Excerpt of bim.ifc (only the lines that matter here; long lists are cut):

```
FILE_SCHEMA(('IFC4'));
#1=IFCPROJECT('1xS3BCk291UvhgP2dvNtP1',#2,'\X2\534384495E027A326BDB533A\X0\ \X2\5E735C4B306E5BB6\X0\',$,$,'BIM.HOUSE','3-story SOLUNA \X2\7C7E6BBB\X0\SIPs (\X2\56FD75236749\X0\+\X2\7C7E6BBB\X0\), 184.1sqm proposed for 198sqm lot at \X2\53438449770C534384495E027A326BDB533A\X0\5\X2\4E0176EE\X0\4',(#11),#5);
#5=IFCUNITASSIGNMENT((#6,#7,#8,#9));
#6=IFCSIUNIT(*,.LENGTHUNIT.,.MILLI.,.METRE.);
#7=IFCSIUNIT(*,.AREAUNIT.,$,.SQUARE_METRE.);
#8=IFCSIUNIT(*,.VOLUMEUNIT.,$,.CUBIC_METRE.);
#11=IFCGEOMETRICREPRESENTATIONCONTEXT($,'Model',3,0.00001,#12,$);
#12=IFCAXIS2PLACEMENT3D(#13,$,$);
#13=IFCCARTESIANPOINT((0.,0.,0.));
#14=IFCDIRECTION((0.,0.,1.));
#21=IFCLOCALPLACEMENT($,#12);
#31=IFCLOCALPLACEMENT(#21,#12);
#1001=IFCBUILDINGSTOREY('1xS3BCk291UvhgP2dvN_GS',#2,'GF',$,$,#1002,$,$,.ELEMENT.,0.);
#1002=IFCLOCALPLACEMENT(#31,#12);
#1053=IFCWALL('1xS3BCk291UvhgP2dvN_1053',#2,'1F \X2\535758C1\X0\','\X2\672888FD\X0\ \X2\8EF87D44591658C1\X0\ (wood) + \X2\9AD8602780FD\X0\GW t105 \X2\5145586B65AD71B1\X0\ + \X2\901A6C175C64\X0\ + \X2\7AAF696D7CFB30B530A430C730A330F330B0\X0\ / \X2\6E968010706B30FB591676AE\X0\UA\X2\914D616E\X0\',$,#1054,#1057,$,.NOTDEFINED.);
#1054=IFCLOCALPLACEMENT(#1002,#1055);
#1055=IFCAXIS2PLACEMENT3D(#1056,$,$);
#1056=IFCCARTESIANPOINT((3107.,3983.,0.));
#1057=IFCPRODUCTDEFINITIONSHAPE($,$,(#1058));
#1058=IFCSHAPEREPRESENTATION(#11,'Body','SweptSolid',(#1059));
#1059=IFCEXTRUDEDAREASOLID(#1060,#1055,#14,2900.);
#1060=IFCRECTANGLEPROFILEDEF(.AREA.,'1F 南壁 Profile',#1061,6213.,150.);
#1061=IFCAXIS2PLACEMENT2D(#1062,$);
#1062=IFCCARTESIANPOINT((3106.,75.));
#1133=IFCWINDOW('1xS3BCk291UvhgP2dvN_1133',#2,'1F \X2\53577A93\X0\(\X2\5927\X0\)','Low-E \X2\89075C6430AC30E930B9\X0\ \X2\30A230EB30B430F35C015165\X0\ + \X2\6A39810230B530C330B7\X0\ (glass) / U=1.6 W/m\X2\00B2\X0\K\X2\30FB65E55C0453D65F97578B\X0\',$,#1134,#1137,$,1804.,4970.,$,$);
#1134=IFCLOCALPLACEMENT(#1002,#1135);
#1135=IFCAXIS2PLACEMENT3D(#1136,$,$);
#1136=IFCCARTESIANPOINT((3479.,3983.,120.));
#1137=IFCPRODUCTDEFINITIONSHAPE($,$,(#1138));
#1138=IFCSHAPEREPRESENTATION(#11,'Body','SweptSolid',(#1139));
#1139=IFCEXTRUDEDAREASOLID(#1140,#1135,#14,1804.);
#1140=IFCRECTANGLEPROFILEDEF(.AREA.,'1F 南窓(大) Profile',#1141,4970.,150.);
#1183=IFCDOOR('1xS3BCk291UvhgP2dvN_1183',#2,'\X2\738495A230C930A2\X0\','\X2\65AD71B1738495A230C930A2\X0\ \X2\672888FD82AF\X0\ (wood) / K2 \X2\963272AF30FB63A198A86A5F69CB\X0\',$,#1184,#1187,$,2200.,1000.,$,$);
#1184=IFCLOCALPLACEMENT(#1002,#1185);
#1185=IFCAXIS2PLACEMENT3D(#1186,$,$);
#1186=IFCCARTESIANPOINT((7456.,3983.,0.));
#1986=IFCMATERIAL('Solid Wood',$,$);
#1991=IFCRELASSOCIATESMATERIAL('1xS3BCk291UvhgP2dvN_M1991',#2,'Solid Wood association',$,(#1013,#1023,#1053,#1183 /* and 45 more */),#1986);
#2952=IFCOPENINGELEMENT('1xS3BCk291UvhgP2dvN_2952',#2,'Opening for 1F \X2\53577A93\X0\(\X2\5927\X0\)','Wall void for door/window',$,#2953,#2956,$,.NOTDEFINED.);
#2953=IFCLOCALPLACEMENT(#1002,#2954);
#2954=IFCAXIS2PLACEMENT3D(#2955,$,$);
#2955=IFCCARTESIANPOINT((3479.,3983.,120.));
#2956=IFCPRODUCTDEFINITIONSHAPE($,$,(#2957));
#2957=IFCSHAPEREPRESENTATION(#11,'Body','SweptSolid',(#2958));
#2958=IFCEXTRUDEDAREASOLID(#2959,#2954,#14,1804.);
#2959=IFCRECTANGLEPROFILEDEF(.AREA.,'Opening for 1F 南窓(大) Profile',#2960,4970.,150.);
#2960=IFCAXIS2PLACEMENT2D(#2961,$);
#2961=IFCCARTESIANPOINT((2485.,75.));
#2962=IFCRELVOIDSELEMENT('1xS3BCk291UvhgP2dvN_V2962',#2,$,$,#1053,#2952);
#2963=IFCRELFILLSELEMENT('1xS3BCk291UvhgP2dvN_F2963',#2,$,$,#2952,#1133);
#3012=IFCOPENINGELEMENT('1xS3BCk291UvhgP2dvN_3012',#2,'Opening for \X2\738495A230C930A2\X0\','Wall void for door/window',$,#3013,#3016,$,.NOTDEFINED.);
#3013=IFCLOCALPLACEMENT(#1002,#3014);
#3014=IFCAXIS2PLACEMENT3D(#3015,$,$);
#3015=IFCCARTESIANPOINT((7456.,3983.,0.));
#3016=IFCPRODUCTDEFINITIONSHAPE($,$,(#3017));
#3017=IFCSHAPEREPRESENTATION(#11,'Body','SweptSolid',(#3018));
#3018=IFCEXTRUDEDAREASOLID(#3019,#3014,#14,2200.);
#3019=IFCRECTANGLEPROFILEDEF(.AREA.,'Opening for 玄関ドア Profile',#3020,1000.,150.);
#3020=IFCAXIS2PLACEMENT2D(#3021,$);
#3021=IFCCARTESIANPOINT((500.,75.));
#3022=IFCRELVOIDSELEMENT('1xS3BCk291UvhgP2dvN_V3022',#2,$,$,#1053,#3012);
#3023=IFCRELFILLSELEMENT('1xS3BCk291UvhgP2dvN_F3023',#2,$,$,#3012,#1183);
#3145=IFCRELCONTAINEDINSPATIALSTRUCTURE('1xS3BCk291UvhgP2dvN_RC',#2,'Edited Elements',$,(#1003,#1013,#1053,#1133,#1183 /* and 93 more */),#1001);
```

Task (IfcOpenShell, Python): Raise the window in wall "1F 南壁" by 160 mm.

```python
import numpy as np
import ifcopenshell
import ifcopenshell.api.geometry
import ifcopenshell.util.placement
import ifcopenshell.util.unit

model = ifcopenshell.open("bim.ifc")
unit_scale = ifcopenshell.util.unit.calculate_unit_scale(model)

window = model.by_guid("1xS3BCk291UvhgP2dvN_1133")
opening = window.FillsVoids[0].RelatingOpeningElement
dz = 160.0

shift = np.array([0.0, 0.0, dz])
# The window is not placed relative to its opening, so move both.
for product in (opening, window):
    matrix = ifcopenshell.util.placement.get_local_placement(product.ObjectPlacement)
    matrix[:3, 3] += shift
    ifcopenshell.api.geometry.edit_object_placement(model, product=product, matrix=matrix, is_si=False)

print(f"moved by {dz * unit_scale:+.3f} m")

model.write("bim_edited.ifc")
```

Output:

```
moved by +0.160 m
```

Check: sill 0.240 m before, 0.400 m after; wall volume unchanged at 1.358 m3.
